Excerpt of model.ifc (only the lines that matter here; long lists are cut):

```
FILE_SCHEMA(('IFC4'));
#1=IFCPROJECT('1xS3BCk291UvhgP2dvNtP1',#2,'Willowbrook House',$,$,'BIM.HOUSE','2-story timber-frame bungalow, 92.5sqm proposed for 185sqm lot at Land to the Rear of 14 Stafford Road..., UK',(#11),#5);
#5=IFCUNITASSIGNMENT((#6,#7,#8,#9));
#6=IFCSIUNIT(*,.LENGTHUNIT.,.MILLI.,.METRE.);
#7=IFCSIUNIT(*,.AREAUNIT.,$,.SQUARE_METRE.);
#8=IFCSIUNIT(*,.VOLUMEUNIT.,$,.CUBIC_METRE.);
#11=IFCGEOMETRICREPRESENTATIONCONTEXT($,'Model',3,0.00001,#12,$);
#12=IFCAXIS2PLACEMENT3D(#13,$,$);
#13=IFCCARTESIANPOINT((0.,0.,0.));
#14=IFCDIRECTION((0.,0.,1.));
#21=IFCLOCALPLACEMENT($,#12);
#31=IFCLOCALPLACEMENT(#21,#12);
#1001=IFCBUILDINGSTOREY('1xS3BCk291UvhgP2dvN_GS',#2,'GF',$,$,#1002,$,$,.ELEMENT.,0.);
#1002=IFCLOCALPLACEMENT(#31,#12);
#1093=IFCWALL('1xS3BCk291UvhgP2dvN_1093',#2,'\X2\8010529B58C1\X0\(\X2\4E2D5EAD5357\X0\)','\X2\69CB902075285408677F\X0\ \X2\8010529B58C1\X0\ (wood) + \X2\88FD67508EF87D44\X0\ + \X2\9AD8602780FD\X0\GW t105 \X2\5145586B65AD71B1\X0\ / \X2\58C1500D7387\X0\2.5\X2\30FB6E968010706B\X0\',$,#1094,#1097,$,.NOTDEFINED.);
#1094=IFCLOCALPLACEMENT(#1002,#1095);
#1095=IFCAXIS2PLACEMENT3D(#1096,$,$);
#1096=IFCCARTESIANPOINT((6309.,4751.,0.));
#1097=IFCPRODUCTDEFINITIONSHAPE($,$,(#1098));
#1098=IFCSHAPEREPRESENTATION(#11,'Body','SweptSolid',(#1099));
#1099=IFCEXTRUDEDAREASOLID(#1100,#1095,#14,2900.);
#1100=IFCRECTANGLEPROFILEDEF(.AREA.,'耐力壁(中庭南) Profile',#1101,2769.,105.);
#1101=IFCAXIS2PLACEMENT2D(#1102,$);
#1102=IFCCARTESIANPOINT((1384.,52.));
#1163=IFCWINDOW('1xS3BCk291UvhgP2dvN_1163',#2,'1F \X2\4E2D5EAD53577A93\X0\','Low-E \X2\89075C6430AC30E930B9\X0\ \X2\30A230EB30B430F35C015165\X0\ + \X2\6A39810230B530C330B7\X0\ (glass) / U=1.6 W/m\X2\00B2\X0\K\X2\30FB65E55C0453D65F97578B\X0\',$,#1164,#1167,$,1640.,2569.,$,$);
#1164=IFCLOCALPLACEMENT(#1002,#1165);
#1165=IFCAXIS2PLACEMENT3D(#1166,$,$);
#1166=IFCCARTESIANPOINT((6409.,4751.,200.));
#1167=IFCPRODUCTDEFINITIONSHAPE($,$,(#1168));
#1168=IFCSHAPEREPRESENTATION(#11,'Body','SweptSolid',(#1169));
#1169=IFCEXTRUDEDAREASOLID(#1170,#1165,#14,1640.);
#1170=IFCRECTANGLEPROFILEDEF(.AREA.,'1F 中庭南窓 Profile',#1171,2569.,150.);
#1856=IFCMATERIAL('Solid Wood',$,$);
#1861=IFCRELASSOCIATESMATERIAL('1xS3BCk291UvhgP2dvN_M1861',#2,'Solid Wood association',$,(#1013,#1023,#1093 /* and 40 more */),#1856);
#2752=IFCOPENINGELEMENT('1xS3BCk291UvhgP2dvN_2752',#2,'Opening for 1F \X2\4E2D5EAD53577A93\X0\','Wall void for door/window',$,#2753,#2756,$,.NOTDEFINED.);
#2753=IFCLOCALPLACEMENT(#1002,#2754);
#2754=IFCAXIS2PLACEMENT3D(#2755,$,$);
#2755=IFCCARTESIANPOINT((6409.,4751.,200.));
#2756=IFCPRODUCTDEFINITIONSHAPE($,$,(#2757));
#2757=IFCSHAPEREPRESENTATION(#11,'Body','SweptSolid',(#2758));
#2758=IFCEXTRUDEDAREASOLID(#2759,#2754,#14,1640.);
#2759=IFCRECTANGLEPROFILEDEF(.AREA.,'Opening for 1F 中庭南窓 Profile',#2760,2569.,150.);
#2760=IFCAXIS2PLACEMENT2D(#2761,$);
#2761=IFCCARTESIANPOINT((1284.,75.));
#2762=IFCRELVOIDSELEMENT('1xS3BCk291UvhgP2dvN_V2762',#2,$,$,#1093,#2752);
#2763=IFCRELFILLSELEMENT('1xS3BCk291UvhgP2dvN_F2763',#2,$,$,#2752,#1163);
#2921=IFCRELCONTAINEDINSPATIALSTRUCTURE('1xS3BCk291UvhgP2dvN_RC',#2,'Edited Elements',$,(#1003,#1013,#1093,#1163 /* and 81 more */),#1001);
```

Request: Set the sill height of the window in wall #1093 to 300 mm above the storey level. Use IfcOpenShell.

```python
import numpy as np
import ifcopenshell
import ifcopenshell.api.geometry
import ifcopenshell.geom
import ifcopenshell.util.element
import ifcopenshell.util.placement
import ifcopenshell.util.shape
import ifcopenshell.util.unit

model = ifcopenshell.open("model.ifc")
unit_scale = ifcopenshell.util.unit.calculate_unit_scale(model)

window = model.by_guid("1xS3BCk291UvhgP2dvN_1163")
opening = window.FillsVoids[0].RelatingOpeningElement
storey = ifcopenshell.util.element.get_container(window, ifc_class="IfcBuildingStorey")
level = ifcopenshell.util.placement.get_local_placement(storey.ObjectPlacement)[2, 3]

# The opening's origin need not be at the sill, so measure its lowest point.
shape = ifcopenshell.geom.create_shape(ifcopenshell.geom.settings(), opening)
bottom = ifcopenshell.util.shape.get_shape_bottom_elevation(shape, shape.geometry) / unit_scale
dz = level + 0.3 / unit_scale - bottom

shift = np.array([0.0, 0.0, dz])
# The window is not placed relative to its opening, so move both.
for product in (opening, window):
    matrix = ifcopenshell.util.placement.get_local_placement(product.ObjectPlacement)
    matrix[:3, 3] += shift
    ifcopenshell.api.geometry.edit_object_placement(model, product=product, matrix=matrix, is_si=False)

print(f"moved by {dz * unit_scale:+.3f} m")

model.write("model_v2.ifc")
```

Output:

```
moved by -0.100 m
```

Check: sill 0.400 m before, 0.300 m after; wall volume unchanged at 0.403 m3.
